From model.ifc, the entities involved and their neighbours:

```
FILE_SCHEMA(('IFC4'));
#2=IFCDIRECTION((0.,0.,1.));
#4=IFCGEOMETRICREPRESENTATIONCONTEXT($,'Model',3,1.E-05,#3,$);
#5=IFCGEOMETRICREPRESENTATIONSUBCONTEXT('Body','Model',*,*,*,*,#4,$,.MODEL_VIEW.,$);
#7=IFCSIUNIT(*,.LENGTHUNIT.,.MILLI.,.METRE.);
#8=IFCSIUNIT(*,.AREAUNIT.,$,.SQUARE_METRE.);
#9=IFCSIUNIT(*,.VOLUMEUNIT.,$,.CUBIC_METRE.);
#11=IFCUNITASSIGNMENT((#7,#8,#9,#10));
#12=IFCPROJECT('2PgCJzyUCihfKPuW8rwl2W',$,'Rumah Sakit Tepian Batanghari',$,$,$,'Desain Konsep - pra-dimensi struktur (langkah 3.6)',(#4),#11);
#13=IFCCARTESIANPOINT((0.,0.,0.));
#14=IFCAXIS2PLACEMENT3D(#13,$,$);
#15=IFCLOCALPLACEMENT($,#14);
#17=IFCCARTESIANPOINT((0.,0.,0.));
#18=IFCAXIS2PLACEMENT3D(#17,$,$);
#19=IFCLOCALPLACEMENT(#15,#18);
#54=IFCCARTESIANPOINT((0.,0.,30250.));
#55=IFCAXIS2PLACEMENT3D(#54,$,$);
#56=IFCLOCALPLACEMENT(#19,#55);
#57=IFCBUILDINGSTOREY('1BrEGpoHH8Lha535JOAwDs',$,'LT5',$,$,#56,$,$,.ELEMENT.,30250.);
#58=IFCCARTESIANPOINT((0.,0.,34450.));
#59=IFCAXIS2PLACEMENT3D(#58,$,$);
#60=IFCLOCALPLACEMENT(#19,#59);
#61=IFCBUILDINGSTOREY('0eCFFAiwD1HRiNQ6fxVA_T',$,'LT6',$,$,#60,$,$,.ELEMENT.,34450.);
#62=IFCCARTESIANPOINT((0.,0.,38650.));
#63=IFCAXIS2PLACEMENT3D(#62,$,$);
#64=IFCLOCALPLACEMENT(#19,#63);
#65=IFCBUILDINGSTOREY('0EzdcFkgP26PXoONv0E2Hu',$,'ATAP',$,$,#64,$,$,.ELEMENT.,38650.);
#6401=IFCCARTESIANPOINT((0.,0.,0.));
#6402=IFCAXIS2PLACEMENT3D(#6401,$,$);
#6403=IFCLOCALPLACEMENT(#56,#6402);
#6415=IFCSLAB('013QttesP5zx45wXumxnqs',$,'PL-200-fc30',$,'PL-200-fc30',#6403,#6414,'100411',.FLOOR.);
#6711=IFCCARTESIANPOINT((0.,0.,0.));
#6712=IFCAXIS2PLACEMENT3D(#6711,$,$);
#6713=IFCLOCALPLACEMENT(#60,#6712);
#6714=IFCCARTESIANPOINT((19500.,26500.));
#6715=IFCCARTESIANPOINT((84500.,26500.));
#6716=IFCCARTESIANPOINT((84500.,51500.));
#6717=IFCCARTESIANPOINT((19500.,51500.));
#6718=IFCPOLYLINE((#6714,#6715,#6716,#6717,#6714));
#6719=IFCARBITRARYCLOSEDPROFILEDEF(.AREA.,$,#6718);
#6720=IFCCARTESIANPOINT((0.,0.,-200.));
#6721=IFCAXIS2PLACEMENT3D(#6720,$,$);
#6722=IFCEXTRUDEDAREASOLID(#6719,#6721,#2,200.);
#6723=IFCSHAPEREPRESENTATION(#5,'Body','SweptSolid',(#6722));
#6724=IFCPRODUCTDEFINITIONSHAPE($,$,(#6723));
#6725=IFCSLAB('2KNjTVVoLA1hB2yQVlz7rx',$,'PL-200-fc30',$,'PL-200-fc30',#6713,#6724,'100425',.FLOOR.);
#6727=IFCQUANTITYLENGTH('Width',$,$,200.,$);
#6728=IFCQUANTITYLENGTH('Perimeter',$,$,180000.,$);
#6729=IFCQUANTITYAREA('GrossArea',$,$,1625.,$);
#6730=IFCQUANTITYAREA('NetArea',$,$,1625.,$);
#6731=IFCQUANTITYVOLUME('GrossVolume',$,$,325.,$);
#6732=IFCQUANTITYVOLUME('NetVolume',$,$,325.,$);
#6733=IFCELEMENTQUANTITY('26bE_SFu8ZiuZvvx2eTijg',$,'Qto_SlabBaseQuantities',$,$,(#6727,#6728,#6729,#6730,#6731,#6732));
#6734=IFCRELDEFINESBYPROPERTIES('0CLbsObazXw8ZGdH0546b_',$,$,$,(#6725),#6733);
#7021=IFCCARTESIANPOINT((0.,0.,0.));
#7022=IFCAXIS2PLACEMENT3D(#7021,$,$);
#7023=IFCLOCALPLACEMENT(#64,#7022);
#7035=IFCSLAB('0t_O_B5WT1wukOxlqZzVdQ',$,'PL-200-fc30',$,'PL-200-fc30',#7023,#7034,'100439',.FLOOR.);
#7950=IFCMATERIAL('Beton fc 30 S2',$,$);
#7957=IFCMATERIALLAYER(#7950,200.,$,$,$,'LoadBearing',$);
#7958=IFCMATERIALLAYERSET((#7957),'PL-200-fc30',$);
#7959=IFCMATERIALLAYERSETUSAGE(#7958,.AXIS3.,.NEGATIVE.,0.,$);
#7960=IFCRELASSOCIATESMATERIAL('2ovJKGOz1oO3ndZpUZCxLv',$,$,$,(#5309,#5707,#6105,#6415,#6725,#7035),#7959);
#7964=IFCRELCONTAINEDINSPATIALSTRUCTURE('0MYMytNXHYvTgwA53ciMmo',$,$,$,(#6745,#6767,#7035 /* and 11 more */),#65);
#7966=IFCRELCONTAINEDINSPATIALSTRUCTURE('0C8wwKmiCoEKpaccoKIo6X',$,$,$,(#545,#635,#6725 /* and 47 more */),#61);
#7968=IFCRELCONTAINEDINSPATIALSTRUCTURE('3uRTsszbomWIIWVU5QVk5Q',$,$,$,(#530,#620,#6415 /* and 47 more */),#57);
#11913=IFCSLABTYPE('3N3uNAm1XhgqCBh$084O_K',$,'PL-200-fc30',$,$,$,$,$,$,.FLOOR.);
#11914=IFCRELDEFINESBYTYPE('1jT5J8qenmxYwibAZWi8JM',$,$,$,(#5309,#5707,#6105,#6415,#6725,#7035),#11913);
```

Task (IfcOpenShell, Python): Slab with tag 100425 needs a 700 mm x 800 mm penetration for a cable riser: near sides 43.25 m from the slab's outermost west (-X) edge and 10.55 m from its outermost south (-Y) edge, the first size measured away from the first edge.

```python
import numpy as np
import ifcopenshell
import ifcopenshell.api.feature
import ifcopenshell.api.geometry
import ifcopenshell.api.pset
import ifcopenshell.api.root
import ifcopenshell.geom
import ifcopenshell.util.element
import ifcopenshell.util.placement
import ifcopenshell.util.representation
import ifcopenshell.util.shape
import ifcopenshell.util.unit

model = ifcopenshell.open("model.ifc")
unit_scale = ifcopenshell.util.unit.calculate_unit_scale(model)
area_scale = ifcopenshell.util.unit.calculate_unit_scale(model, "AREAUNIT")
volume_scale = ifcopenshell.util.unit.calculate_unit_scale(model, "VOLUMEUNIT")
settings = ifcopenshell.geom.settings()


def volume(element):
    """Net volume in cubic metres, openings subtracted."""
    shape = ifcopenshell.geom.create_shape(settings, element)
    return ifcopenshell.util.shape.get_volume(shape.geometry)


slab = model.by_guid("2KNjTVVoLA1hB2yQVlz7rx")
before = volume(slab)

# Extent in the slab's own axes, in metres. The edges named are its -X and -Y sides.
slab_shape = ifcopenshell.geom.create_shape(settings, slab)
vertices = ifcopenshell.util.shape.get_vertices(slab_shape.geometry)
x_min, y_min, bottom = vertices.min(axis=0)
top = vertices[:, 2].max()

opening = ifcopenshell.api.root.create_entity(model, ifc_class="IfcOpeningElement", name="Cable riser opening", predefined_type="OPENING")
context = ifcopenshell.util.representation.get_context(model, "Model", "Body", "MODEL_VIEW")
width, depth = 0.7, 0.8
outline = [(0.0, 0.0), (width, 0.0), (width, depth), (0.0, depth), (0.0, 0.0)]
# Overshoot both faces by 50 mm so the cut is clean.
shape = ifcopenshell.api.geometry.add_slab_representation(
    model, context=context, depth=top - bottom + 0.1, polyline=outline
)
ifcopenshell.api.geometry.assign_representation(model, product=opening, representation=shape)

matrix = ifcopenshell.util.placement.get_local_placement(slab.ObjectPlacement)
matrix[:, 3] = matrix @ np.append(np.array([x_min + 43.25, y_min + 10.55, bottom - 0.05]) / unit_scale, 1.0)
ifcopenshell.api.geometry.edit_object_placement(model, product=opening, matrix=matrix, is_si=False)
ifcopenshell.api.feature.add_feature(model, feature=opening, element=slab)

after = volume(slab)

# Update the slab's stored quantities.
qto = model.by_id(ifcopenshell.util.element.get_pset(slab, "Qto_SlabBaseQuantities", should_inherit=False)["id"])
ifcopenshell.api.pset.edit_qto(model, qto=qto, properties={
    "NetArea": after / (top - bottom) / area_scale,
    "NetVolume": after / volume_scale,
})

print(f"slab volume {before:.3f} -> {after:.3f} m3")

model.write("model_edited.ifc")
```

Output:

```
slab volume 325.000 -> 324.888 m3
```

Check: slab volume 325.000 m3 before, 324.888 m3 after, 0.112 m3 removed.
